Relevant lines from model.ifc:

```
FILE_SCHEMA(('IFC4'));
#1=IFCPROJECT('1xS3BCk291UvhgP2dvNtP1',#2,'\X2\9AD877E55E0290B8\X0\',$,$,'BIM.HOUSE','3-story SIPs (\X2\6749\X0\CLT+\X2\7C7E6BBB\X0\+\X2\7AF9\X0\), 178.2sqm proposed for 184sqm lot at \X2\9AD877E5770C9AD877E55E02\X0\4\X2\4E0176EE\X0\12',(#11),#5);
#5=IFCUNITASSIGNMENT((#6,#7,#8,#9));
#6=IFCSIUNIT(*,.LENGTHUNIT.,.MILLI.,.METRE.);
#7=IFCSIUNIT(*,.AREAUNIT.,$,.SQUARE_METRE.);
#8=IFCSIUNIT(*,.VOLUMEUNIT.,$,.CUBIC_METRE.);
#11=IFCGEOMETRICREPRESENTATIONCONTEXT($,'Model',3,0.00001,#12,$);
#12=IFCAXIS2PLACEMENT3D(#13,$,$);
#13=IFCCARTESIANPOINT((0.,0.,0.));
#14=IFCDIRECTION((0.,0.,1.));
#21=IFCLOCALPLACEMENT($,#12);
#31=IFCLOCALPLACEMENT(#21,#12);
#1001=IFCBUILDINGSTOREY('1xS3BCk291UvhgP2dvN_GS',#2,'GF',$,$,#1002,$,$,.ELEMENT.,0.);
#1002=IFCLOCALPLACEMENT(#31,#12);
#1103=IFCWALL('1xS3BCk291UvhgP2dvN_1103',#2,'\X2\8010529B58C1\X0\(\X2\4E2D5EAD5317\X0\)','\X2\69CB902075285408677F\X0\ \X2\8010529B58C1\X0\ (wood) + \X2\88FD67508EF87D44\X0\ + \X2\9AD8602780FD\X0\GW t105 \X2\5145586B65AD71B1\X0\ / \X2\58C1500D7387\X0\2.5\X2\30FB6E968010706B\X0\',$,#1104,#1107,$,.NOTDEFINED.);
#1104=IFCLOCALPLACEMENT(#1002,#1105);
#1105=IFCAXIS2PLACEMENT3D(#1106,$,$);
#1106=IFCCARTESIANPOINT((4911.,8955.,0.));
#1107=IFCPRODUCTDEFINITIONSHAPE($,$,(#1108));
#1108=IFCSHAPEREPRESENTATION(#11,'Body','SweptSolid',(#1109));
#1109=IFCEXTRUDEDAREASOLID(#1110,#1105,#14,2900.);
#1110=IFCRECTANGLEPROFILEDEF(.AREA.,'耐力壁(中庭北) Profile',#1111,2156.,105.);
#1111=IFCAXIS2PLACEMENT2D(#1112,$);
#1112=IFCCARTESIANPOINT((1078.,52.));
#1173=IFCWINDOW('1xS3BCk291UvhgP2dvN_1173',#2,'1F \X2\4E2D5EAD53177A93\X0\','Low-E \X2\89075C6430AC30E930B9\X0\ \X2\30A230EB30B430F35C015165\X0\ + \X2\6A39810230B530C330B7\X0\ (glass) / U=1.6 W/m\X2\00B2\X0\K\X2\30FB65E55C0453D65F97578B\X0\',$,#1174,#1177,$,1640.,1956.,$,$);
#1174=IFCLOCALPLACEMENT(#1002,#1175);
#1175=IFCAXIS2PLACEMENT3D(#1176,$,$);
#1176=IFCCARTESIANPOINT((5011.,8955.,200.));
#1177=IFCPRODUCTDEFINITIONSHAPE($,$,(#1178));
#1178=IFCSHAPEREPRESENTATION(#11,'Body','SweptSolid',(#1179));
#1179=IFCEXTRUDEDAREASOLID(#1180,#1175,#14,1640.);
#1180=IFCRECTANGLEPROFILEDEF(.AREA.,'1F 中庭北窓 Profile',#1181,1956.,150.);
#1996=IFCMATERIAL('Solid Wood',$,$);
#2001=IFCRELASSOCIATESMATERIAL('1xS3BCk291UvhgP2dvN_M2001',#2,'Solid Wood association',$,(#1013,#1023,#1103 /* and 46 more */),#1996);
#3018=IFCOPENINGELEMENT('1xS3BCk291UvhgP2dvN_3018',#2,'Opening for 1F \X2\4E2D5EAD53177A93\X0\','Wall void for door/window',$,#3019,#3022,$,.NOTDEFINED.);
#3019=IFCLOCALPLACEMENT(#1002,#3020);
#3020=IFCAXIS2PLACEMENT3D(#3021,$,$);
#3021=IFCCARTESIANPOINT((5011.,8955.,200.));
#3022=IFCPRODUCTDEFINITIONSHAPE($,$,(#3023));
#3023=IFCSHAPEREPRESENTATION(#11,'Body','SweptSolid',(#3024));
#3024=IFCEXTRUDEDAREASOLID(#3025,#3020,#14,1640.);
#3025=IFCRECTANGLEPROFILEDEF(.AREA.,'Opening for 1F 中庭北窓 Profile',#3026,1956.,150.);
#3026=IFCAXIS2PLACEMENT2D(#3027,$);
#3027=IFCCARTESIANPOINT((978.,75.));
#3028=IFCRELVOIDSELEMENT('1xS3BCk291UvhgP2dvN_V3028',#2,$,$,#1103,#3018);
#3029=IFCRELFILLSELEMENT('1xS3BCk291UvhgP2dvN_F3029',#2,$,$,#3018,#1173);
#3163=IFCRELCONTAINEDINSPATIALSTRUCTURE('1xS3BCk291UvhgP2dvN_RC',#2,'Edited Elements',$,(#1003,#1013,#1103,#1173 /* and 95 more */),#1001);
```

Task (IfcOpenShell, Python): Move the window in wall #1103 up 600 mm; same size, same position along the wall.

```python
import numpy as np
import ifcopenshell
import ifcopenshell.api.geometry
import ifcopenshell.util.placement
import ifcopenshell.util.unit

model = ifcopenshell.open("model.ifc")
unit_scale = ifcopenshell.util.unit.calculate_unit_scale(model)

window = model.by_guid("1xS3BCk291UvhgP2dvN_1173")
opening = window.FillsVoids[0].RelatingOpeningElement
dz = 0.6 / unit_scale

shift = np.array([0.0, 0.0, dz])
# The window is not placed relative to its opening, so move both.
for product in (opening, window):
    matrix = ifcopenshell.util.placement.get_local_placement(product.ObjectPlacement)
    matrix[:3, 3] += shift
    ifcopenshell.api.geometry.edit_object_placement(model, product=product, matrix=matrix, is_si=False)

print(f"moved by {dz * unit_scale:+.3f} m")

model.write("model_rev.ifc")
```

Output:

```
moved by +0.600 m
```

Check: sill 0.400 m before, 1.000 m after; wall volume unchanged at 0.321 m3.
